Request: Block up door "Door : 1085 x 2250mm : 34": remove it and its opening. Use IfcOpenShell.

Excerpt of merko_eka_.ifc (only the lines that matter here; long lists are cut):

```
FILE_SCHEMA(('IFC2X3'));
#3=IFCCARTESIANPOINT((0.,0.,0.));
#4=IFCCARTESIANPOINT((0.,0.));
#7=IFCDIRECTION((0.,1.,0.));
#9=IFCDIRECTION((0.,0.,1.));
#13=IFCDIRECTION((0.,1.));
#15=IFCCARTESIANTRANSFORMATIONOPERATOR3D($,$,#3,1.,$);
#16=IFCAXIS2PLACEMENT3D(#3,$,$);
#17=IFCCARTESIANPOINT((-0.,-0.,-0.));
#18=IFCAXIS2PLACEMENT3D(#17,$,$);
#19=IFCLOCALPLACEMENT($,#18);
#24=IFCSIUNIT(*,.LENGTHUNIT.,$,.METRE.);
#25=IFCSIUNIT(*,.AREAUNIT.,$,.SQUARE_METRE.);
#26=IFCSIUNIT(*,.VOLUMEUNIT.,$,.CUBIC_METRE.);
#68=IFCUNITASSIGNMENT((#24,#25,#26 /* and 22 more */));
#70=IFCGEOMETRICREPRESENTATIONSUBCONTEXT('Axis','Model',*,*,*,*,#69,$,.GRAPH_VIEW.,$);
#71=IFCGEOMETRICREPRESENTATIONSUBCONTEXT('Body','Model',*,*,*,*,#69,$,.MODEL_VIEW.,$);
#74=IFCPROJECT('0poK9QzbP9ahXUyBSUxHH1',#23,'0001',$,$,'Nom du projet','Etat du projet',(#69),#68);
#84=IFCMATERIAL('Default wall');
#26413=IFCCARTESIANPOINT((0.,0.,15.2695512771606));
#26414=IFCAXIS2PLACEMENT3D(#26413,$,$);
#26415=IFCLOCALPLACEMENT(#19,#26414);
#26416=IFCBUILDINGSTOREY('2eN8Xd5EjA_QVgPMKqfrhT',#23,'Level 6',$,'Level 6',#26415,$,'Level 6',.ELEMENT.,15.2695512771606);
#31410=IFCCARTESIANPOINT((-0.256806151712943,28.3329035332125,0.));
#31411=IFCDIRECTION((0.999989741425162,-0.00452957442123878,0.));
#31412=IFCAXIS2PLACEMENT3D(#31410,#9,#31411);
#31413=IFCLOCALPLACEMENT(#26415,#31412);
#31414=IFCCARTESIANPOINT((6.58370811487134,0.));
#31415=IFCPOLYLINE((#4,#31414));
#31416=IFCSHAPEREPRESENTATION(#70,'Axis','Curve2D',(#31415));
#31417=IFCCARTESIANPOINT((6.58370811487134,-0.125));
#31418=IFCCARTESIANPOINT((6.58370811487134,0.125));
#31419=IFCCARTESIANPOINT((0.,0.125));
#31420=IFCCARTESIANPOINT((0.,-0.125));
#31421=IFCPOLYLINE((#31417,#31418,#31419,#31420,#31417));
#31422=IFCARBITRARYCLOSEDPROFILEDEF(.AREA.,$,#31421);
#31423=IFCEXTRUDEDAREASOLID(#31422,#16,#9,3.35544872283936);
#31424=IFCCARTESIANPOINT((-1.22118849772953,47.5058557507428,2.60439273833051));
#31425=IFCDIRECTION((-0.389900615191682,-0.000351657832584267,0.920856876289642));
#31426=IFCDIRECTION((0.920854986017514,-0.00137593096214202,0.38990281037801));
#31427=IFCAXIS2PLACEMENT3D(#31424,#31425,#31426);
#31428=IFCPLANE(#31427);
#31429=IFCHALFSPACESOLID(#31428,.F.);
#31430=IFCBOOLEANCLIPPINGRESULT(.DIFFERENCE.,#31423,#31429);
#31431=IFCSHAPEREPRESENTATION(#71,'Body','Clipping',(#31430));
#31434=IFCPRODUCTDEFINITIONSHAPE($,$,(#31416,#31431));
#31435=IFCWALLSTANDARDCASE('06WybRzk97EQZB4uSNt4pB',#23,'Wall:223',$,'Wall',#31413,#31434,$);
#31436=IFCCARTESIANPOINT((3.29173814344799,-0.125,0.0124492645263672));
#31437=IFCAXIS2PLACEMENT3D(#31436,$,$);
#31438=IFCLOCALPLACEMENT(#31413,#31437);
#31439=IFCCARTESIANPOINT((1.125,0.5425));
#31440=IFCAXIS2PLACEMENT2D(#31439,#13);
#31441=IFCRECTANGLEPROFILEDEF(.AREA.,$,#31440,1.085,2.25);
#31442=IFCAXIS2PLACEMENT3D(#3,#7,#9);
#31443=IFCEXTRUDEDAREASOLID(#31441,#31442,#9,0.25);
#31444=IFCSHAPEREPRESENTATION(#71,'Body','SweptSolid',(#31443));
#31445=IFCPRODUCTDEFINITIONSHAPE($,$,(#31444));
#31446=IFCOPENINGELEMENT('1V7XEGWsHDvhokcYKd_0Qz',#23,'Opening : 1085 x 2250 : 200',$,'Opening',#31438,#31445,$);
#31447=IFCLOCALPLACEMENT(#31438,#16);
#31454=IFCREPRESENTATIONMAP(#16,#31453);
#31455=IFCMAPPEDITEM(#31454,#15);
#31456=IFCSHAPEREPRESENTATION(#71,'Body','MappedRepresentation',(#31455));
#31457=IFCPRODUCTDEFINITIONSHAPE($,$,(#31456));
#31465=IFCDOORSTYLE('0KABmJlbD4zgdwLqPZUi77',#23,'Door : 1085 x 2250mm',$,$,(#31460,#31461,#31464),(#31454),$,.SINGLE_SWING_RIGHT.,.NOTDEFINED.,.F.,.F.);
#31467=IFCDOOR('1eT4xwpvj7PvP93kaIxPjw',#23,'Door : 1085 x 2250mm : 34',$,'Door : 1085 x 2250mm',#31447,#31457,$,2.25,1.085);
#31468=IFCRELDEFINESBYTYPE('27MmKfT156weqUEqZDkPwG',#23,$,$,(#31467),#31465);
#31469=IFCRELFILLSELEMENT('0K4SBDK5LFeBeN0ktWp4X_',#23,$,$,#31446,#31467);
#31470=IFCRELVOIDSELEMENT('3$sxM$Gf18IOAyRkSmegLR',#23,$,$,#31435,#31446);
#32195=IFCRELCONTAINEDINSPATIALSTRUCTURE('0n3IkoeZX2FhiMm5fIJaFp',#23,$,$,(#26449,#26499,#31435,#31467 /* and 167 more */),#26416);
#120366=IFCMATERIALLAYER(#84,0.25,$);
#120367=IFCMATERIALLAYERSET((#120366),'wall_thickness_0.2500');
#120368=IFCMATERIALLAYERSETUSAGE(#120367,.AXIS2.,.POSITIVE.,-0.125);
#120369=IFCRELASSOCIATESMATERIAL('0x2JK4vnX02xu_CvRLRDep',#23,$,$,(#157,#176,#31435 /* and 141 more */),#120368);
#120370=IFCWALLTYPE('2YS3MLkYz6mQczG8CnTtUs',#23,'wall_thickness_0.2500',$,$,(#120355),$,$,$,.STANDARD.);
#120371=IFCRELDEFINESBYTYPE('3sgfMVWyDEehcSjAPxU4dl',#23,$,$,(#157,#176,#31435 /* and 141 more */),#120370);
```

```python
import ifcopenshell
import ifcopenshell.api.feature
import ifcopenshell.api.root
import ifcopenshell.geom
import ifcopenshell.util.shape

model = ifcopenshell.open("merko_eka_.ifc")
settings = ifcopenshell.geom.settings()


def volume(element):
    """Net volume in cubic metres, openings subtracted."""
    shape = ifcopenshell.geom.create_shape(settings, element)
    return ifcopenshell.util.shape.get_volume(shape.geometry)


door = model.by_guid("1eT4xwpvj7PvP93kaIxPjw")
opening = door.FillsVoids[0].RelatingOpeningElement
wall = opening.VoidsElements[0].RelatingBuildingElement
before = volume(wall)

ifcopenshell.api.root.remove_product(model, product=door)
ifcopenshell.api.feature.remove_feature(model, feature=opening)

after = volume(wall)

print(f"wall volume {before:.3f} -> {after:.3f} m3")

model.write("merko_eka__rev.ifc")
```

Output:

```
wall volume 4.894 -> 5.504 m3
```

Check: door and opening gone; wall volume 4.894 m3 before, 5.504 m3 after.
